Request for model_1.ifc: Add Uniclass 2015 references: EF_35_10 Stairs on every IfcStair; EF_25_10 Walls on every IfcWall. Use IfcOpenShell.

First a look at what the model holds.

```python
import ifcopenshell

model = ifcopenshell.open("model_1.ifc")
print(model.schema)
print("classifications:", [c.Name for c in model.by_type("IfcClassification")])
for ifc_class in ("IfcDoor", "IfcRoof", "IfcStair", "IfcWall", "IfcWindow"):
    print(ifc_class, len(model.by_type(ifc_class)))
```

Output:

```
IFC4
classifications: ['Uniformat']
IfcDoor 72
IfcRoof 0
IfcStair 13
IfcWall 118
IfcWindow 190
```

```python
import ifcopenshell
import ifcopenshell.api.classification

model = ifcopenshell.open("model_1.ifc")

system = ifcopenshell.api.classification.add_classification(model, classification="Uniclass 2015")

codes = {
    "IfcStair": ("EF_35_10", "Stairs"),
    "IfcWall": ("EF_25_10", "Walls"),
}
for ifc_class, (code, name) in codes.items():
    products = model.by_type(ifc_class)
    ifcopenshell.api.classification.add_reference(
        model, products=products, classification=system, identification=code, name=name
    )
    print(code, len(products))

model.write("model_1-out.ifc")
```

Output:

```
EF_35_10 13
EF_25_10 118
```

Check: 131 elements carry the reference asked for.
